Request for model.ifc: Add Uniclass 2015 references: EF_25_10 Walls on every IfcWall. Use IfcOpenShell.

First a look at what the model holds.

```python
import ifcopenshell

model = ifcopenshell.open("model.ifc")
print(model.schema)
print("classifications:", [c.Name for c in model.by_type("IfcClassification")])
for ifc_class in ("IfcDoor", "IfcRoof", "IfcStair", "IfcWall", "IfcWindow"):
    print(ifc_class, len(model.by_type(ifc_class)))
```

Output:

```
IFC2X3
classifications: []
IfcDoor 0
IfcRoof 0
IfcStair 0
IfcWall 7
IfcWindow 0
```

```python
import ifcopenshell
import ifcopenshell.api.classification

model = ifcopenshell.open("model.ifc")

# IFC2X3 requires Source and Edition and has no link from the project to the system.
system = model.create_entity("IfcClassification", Source="NBS", Edition="2015", Name="Uniclass 2015")

codes = {
    "IfcWall": ("EF_25_10", "Walls"),
}
for ifc_class, (code, name) in codes.items():
    products = model.by_type(ifc_class)
    ifcopenshell.api.classification.add_reference(
        model, products=products, classification=system, identification=code, name=name
    )
    print(code, len(products))

model.write("model_updated.ifc")
```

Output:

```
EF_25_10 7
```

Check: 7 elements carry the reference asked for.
